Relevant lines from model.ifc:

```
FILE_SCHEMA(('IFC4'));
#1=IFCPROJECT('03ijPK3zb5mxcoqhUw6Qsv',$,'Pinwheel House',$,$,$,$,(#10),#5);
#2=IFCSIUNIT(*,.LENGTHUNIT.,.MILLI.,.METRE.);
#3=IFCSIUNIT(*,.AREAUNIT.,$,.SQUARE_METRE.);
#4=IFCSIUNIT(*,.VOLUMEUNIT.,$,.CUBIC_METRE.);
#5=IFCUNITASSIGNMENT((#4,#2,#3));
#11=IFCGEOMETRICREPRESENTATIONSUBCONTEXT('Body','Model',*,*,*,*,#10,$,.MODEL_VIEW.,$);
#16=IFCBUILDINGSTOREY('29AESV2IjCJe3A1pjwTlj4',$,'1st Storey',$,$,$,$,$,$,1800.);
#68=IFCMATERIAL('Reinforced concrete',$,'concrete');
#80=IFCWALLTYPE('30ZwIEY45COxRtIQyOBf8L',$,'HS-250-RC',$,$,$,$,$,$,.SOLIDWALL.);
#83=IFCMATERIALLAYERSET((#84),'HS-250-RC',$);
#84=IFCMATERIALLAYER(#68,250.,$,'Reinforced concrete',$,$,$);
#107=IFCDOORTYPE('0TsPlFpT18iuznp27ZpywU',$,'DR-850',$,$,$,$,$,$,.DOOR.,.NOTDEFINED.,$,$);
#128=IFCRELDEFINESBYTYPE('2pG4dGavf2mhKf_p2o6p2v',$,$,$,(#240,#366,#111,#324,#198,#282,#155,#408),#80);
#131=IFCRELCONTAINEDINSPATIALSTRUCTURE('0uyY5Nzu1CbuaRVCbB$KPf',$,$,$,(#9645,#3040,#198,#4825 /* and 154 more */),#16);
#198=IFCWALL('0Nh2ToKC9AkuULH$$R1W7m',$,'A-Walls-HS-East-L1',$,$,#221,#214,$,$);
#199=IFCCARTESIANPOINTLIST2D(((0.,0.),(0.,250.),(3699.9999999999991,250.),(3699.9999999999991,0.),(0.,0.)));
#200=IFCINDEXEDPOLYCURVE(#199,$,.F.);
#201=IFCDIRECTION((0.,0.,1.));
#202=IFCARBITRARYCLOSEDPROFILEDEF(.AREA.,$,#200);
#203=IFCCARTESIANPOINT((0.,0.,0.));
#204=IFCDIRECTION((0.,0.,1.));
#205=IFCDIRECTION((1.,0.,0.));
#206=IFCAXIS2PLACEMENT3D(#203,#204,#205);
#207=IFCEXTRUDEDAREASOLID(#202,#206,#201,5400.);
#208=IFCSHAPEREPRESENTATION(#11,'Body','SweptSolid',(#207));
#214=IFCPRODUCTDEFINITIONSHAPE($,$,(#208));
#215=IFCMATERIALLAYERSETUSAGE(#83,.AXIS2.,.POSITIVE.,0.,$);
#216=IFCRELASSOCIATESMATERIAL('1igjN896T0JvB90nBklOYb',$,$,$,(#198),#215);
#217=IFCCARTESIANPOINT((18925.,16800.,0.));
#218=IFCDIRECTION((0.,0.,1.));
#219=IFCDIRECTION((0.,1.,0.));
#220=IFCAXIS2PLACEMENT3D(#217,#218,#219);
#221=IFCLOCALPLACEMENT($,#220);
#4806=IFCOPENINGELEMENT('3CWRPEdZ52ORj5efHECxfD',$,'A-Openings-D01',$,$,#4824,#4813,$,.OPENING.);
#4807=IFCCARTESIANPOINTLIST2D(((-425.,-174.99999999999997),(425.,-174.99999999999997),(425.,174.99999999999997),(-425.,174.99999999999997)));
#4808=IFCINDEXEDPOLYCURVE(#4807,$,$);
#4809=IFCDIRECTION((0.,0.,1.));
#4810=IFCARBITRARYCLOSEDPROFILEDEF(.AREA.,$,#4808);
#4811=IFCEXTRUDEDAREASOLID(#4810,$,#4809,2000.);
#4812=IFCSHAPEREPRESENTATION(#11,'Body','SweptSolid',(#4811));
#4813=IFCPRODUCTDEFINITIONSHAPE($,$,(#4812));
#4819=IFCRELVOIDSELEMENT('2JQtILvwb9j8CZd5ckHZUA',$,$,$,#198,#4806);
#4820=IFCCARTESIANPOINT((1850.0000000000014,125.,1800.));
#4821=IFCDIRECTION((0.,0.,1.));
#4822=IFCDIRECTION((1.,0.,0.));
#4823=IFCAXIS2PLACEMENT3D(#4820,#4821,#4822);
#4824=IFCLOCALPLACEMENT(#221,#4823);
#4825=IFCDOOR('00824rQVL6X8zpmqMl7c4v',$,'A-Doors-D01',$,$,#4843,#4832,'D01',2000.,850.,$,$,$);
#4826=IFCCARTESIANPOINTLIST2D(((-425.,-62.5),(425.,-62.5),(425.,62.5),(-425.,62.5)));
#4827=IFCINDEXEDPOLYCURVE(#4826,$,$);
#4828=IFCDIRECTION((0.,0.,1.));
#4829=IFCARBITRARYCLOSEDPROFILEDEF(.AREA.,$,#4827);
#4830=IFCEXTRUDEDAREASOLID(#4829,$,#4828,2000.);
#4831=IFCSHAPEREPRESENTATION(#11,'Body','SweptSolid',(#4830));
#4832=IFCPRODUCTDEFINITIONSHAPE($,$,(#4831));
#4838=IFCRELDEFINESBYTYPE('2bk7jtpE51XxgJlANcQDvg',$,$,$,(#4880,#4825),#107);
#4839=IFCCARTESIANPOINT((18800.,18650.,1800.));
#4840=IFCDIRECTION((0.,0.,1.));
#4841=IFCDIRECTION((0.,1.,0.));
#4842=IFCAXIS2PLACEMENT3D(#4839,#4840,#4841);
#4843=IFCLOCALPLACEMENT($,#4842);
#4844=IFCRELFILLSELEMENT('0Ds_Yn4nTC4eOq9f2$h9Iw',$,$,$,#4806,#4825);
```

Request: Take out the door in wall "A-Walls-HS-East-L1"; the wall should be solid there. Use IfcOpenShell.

```python
import ifcopenshell
import ifcopenshell.api.feature
import ifcopenshell.api.root
import ifcopenshell.geom
import ifcopenshell.util.shape

model = ifcopenshell.open("model.ifc")
settings = ifcopenshell.geom.settings()


def volume(element):
    """Net volume in cubic metres, openings subtracted."""
    shape = ifcopenshell.geom.create_shape(settings, element)
    return ifcopenshell.util.shape.get_volume(shape.geometry)


door = model.by_id(4825)
opening = door.FillsVoids[0].RelatingOpeningElement
wall = opening.VoidsElements[0].RelatingBuildingElement
before = volume(wall)

ifcopenshell.api.root.remove_product(model, product=door)
ifcopenshell.api.feature.remove_feature(model, feature=opening)

after = volume(wall)

print(f"wall volume {before:.3f} -> {after:.3f} m3")

model.write("model_updated.ifc")
```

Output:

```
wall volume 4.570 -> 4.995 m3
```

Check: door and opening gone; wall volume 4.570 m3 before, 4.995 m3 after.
